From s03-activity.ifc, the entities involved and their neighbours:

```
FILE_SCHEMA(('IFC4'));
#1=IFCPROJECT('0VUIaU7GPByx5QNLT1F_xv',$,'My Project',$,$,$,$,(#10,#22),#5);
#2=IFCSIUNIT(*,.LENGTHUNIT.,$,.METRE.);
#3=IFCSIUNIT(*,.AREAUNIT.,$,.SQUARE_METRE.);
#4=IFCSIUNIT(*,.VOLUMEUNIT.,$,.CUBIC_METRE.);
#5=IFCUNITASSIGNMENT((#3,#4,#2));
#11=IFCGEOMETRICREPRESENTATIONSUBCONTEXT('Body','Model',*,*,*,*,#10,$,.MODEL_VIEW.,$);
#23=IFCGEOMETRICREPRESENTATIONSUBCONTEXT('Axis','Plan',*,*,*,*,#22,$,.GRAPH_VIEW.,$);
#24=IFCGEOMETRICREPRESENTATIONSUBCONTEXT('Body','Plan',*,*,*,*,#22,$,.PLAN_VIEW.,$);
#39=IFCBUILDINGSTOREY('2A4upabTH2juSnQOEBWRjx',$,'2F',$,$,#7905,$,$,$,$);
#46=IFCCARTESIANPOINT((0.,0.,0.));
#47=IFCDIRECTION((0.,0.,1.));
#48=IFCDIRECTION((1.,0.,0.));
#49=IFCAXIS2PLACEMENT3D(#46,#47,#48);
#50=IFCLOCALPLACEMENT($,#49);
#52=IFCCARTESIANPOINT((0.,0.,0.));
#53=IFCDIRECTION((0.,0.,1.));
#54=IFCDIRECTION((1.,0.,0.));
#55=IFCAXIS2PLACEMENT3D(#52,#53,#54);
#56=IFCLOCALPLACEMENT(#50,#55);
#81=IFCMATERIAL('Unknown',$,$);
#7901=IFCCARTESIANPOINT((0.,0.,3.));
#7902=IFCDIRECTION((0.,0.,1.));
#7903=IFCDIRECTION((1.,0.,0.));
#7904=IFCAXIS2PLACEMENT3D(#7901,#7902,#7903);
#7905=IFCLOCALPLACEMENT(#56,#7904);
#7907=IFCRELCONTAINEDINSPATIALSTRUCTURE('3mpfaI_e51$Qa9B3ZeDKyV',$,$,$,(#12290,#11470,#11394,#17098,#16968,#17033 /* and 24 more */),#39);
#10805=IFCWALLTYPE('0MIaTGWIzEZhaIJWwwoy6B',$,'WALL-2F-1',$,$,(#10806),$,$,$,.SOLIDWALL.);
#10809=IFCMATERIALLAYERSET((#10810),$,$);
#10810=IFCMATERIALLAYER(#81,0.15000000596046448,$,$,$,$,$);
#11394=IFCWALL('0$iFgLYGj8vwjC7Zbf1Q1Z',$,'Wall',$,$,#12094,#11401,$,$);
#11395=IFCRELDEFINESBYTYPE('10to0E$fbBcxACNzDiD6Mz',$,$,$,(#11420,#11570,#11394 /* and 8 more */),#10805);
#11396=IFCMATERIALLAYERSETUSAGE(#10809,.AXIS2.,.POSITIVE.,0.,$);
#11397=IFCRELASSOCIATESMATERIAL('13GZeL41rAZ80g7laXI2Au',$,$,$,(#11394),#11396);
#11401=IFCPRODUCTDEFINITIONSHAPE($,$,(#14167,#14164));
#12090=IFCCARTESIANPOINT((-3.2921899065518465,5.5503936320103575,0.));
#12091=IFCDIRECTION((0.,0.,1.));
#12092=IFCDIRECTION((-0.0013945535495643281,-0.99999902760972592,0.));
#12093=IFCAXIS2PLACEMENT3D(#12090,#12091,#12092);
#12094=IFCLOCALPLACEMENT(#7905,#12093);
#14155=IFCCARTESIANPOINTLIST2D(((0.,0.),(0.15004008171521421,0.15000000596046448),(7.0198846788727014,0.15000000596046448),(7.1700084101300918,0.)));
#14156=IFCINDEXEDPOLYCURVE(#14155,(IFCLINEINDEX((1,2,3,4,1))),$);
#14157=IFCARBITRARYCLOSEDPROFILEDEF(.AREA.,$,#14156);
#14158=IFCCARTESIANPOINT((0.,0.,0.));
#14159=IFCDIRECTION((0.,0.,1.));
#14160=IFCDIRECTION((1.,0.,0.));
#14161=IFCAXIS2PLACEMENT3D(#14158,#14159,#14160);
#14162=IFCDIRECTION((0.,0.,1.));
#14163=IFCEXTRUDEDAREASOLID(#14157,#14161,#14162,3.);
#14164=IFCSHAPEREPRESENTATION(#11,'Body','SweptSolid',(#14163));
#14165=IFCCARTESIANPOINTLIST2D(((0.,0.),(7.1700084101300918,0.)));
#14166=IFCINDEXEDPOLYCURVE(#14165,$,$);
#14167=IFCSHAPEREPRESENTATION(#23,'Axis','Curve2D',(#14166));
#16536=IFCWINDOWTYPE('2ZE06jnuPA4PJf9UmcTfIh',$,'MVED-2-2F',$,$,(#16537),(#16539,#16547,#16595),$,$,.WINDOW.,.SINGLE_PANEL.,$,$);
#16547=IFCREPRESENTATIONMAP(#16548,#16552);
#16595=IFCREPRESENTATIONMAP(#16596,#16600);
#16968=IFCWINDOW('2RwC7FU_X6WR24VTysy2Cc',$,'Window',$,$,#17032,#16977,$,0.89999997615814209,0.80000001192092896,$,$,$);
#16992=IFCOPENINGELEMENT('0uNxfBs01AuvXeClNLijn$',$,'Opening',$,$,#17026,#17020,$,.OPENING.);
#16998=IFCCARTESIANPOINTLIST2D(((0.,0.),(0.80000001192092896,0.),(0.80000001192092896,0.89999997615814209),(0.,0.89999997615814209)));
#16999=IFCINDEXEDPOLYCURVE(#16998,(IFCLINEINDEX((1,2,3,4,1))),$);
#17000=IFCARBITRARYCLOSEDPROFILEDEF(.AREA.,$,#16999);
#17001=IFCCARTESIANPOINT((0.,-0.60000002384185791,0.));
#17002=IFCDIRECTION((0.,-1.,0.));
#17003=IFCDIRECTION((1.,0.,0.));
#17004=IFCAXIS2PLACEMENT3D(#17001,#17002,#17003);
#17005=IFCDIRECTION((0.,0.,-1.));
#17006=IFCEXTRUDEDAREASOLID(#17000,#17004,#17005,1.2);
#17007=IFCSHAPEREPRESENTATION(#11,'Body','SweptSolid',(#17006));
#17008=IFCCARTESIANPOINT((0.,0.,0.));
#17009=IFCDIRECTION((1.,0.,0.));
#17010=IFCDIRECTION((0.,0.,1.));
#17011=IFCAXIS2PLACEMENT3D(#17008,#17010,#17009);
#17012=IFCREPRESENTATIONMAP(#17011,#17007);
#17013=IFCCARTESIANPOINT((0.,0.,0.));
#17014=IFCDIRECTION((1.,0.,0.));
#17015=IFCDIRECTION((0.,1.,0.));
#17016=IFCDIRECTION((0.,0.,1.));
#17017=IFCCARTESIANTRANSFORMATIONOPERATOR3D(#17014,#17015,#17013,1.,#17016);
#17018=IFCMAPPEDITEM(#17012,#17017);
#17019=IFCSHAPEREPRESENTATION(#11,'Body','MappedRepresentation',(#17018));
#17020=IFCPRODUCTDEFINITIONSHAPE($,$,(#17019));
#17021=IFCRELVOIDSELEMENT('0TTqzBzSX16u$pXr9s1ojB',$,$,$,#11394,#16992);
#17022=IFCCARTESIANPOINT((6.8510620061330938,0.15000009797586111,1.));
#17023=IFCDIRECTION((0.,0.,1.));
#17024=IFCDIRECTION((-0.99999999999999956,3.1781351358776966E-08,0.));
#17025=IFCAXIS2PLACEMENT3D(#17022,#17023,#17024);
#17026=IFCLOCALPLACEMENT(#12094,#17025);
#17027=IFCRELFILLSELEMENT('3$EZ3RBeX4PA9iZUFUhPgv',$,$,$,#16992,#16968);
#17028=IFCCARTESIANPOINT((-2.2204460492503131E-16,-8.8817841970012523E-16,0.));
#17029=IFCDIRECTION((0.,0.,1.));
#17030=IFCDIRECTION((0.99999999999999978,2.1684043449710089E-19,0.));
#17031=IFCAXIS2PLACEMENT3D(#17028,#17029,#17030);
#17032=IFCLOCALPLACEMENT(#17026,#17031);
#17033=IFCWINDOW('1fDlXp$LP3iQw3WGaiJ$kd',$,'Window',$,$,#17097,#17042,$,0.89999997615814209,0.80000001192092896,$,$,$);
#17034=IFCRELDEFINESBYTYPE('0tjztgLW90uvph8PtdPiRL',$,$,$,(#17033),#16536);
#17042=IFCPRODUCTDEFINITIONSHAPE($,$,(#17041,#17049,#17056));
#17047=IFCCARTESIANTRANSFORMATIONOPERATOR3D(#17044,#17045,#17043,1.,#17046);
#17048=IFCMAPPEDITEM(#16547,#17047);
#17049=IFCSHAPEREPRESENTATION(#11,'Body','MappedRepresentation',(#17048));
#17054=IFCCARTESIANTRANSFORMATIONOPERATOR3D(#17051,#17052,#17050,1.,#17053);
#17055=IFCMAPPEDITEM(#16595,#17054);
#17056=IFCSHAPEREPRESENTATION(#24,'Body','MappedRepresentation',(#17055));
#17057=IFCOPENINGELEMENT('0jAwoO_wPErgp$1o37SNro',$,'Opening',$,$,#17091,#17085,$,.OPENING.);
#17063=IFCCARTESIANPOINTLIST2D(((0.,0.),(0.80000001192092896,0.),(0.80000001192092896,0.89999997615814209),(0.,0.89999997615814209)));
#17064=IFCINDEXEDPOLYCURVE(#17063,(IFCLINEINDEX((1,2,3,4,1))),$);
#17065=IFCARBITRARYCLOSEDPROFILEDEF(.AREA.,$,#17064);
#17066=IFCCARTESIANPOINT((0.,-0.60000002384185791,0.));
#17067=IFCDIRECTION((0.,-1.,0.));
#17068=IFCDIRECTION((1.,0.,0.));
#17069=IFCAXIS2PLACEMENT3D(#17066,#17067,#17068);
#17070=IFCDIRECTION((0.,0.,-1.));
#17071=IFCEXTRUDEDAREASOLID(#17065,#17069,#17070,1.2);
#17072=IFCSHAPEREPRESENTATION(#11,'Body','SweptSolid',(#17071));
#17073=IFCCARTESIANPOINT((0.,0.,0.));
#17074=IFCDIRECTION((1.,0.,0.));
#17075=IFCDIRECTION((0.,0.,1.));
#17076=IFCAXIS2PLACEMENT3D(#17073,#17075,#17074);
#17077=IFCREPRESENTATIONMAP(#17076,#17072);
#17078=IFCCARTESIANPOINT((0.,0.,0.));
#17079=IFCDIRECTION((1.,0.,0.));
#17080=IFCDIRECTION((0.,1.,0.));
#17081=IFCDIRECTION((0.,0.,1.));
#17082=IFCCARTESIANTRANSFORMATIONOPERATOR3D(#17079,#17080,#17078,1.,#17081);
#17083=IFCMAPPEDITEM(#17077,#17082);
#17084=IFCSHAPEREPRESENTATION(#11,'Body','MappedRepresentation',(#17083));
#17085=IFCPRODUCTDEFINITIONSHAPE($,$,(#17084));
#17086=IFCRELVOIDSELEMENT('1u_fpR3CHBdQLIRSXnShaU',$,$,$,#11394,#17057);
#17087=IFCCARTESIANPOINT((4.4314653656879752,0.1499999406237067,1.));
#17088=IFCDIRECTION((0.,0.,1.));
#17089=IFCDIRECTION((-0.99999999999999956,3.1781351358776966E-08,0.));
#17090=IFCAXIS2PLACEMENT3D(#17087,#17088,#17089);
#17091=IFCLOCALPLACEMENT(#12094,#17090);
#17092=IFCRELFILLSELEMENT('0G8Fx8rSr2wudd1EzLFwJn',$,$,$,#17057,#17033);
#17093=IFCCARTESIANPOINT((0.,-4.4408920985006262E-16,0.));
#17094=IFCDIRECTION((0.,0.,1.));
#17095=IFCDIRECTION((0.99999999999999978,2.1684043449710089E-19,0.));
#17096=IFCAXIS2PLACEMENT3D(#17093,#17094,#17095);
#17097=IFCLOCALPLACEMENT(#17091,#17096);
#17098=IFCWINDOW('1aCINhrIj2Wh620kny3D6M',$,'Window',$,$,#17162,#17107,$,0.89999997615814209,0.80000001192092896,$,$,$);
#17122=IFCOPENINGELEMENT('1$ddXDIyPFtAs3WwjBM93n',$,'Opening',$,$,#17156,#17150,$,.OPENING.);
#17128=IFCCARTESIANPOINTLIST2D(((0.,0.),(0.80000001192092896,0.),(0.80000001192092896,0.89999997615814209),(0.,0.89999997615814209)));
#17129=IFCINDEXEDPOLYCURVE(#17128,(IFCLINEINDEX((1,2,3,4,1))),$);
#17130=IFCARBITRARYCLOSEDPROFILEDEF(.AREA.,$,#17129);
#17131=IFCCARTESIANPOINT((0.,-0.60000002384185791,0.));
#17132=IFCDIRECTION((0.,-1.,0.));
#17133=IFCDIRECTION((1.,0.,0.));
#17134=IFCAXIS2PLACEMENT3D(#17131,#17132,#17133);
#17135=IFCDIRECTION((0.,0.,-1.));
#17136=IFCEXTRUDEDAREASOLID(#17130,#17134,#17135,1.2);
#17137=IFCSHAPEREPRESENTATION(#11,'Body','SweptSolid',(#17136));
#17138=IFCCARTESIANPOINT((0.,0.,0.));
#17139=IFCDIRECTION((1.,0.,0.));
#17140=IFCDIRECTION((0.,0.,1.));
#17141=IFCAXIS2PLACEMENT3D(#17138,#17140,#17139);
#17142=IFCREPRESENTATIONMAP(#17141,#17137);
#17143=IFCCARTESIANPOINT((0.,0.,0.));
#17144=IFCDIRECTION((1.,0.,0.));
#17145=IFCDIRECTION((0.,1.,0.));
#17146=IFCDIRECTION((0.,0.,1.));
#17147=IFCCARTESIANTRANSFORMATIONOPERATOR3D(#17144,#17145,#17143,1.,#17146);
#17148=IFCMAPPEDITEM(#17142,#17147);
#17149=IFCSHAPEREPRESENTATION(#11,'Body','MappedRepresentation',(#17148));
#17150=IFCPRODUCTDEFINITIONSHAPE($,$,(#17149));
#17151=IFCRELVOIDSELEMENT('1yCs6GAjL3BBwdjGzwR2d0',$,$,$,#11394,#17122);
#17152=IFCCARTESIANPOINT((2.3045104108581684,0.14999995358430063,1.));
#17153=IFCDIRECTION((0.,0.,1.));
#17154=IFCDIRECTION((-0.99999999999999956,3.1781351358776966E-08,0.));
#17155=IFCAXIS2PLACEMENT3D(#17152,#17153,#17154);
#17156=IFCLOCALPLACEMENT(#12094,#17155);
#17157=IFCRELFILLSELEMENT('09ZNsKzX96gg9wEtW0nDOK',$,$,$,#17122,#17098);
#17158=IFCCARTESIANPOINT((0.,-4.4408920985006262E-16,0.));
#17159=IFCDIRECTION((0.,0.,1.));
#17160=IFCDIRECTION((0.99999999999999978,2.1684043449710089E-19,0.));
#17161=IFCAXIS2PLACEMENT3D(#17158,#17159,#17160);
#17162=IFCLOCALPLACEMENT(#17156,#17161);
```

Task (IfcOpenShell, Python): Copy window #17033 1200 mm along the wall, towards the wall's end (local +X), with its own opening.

```python
import ifcopenshell
import ifcopenshell.api.feature
import ifcopenshell.api.geometry
import ifcopenshell.api.root
import ifcopenshell.geom
import ifcopenshell.util.element
import ifcopenshell.util.placement
import ifcopenshell.util.shape

model = ifcopenshell.open("s03-activity.ifc")
settings = ifcopenshell.geom.settings()


def volume(element):
    """Net volume in cubic metres, openings subtracted."""
    shape = ifcopenshell.geom.create_shape(settings, element)
    return ifcopenshell.util.shape.get_volume(shape.geometry)


window = model.by_guid("1fDlXp$LP3iQw3WGaiJ$kd")
opening = window.FillsVoids[0].RelatingOpeningElement
wall = opening.VoidsElements[0].RelatingBuildingElement
before = volume(wall)
shift = ifcopenshell.util.placement.get_local_placement(wall.ObjectPlacement)[:3, 0] * 1.2

# copy_class copies the void relationship, type, container and properties, but no geometry.
new_opening = ifcopenshell.api.root.copy_class(model, product=opening)
new_opening.Representation = ifcopenshell.util.element.copy_deep(
    model, opening.Representation, exclude=["IfcGeometricRepresentationContext", "IfcRepresentationMap"]
)
new_window = ifcopenshell.api.root.copy_class(model, product=window)
new_window.Representation = ifcopenshell.util.element.copy_deep(
    model, window.Representation, exclude=["IfcGeometricRepresentationContext", "IfcRepresentationMap"]
)
ifcopenshell.api.feature.add_filling(model, opening=new_opening, element=new_window)

for old, new in ((opening, new_opening), (window, new_window)):
    matrix = ifcopenshell.util.placement.get_local_placement(old.ObjectPlacement)
    matrix[:3, 3] += shift
    ifcopenshell.api.geometry.edit_object_placement(model, product=new, matrix=matrix, is_si=False)

after = volume(wall)

print(f"wall volume {before:.3f} -> {after:.3f} m3")

model.write("s03-activity_edited.ifc")
```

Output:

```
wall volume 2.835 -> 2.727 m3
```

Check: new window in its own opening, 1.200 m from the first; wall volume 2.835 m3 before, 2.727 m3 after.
